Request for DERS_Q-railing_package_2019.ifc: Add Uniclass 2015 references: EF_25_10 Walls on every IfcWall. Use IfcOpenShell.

First a look at what the model holds.

```python
import ifcopenshell

model = ifcopenshell.open("DERS_Q-railing_package_2019.ifc")
print(model.schema)
print("classifications:", [c.Name for c in model.by_type("IfcClassification")])
for ifc_class in ("IfcDoor", "IfcRoof", "IfcStair", "IfcWall", "IfcWindow"):
    print(ifc_class, len(model.by_type(ifc_class)))
```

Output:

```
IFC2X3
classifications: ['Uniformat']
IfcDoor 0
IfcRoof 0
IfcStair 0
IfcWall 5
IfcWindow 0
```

```python
import ifcopenshell
import ifcopenshell.api.classification

model = ifcopenshell.open("DERS_Q-railing_package_2019.ifc")

# IFC2X3 requires Source and Edition and has no link from the project to the system.
system = model.create_entity("IfcClassification", Source="NBS", Edition="2015", Name="Uniclass 2015")

codes = {
    "IfcWall": ("EF_25_10", "Walls"),
}
for ifc_class, (code, name) in codes.items():
    products = model.by_type(ifc_class)
    ifcopenshell.api.classification.add_reference(
        model, products=products, classification=system, identification=code, name=name
    )
    print(code, len(products))

model.write("DERS_Q-railing_package_2019_edited.ifc")
```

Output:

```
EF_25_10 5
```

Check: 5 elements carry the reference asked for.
